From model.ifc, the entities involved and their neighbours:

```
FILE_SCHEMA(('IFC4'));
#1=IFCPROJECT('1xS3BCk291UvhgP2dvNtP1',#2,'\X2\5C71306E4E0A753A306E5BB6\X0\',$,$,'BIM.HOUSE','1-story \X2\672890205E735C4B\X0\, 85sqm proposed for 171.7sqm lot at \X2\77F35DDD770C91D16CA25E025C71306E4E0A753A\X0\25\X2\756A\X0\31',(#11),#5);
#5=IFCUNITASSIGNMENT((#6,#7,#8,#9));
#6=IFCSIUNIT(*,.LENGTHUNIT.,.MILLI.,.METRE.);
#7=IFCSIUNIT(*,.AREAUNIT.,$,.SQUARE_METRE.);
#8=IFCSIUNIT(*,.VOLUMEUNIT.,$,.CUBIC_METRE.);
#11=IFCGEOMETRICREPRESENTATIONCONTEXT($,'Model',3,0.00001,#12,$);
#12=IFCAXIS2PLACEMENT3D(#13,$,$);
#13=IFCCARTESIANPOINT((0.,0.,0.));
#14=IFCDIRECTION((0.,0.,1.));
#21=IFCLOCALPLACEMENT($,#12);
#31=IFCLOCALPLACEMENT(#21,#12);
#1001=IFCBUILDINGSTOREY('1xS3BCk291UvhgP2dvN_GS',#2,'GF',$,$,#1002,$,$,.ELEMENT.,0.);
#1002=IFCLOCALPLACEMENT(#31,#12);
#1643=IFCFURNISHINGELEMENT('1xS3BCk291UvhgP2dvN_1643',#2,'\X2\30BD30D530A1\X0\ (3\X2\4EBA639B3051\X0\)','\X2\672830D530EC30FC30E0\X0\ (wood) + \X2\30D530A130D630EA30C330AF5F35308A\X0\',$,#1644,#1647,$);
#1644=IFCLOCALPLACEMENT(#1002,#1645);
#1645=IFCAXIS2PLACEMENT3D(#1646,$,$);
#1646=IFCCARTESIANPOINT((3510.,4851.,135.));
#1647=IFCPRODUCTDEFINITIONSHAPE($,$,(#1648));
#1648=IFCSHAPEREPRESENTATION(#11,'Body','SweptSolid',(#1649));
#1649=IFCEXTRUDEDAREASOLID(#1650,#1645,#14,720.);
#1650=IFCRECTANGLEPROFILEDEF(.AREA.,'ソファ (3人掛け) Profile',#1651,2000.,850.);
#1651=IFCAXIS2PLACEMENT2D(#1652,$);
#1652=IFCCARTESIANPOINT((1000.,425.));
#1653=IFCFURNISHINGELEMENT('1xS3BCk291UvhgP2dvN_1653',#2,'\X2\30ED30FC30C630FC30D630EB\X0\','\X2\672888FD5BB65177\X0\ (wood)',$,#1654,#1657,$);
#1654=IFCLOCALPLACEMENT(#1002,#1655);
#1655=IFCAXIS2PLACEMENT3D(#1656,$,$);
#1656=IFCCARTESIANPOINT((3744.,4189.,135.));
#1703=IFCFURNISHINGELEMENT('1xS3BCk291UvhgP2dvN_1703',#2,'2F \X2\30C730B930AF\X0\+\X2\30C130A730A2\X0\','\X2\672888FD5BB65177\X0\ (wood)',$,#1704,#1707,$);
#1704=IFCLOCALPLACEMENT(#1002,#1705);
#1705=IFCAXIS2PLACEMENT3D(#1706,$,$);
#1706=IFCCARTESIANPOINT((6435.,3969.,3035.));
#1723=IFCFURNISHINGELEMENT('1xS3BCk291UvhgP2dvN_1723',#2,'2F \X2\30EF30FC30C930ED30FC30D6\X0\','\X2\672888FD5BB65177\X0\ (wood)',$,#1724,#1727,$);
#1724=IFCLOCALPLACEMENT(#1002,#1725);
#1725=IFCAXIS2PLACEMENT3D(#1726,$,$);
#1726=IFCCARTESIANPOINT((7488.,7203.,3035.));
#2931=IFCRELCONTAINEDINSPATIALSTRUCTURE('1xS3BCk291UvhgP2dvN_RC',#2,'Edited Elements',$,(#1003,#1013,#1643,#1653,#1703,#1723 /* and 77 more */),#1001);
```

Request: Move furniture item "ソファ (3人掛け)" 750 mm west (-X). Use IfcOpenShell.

```python
import ifcopenshell
import ifcopenshell.api.geometry
import ifcopenshell.util.placement

model = ifcopenshell.open("model.ifc")

item = model.by_id(1643)
matrix = ifcopenshell.util.placement.get_local_placement(item.ObjectPlacement)
matrix[0, 3] -= 750.0
ifcopenshell.api.geometry.edit_object_placement(model, product=item, matrix=matrix, is_si=False)

print(ifcopenshell.util.placement.get_local_placement(item.ObjectPlacement).round(3) + 0.0)

model.write("model_v2.ifc")
```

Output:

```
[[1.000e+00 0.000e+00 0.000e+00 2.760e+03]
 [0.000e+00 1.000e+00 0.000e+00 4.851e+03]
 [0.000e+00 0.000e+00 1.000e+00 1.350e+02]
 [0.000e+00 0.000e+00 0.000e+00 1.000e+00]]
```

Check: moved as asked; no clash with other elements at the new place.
